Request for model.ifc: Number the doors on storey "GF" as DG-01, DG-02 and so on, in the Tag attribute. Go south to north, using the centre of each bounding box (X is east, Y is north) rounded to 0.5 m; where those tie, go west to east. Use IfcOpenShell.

First a look at what the model holds.

```python
import ifcopenshell
import ifcopenshell.util.element
import ifcopenshell.util.placement

model = ifcopenshell.open("model.ifc")
print(model.schema)
storey = next(s for s in model.by_type("IfcBuildingStorey") if s.Name == "GF")
doors = [e for e in ifcopenshell.util.element.get_decomposition(storey) if e.is_a("IfcDoor")]
for e in sorted(doors, key=lambda e: e.id()):
    origin = ifcopenshell.util.placement.get_local_placement(e.ObjectPlacement)[:3, 3]
    print(e.id(), e.Tag, e.Name, origin.round(2) + 0.0, sep=" | ")
```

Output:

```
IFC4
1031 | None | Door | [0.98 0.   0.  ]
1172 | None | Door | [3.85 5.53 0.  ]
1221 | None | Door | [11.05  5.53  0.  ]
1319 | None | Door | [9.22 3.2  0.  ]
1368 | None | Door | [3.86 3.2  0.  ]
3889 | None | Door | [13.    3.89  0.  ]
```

```python
import ifcopenshell
import ifcopenshell.geom
import ifcopenshell.util.element
import ifcopenshell.util.shape

model = ifcopenshell.open("model.ifc")
settings = ifcopenshell.geom.settings()
settings.set("use-world-coords", True)


def centre(element):
    shape = ifcopenshell.geom.create_shape(settings, element)
    return ifcopenshell.util.shape.get_bbox_centroid(shape.geometry)


storey = next(s for s in model.by_type("IfcBuildingStorey") if s.Name == "GF")
doors = [e for e in ifcopenshell.util.element.get_decomposition(storey) if e.is_a("IfcDoor")]

# Insertion points can sit at a corner or the storey origin, so sort by the geometry (in metres).
centres = {e: centre(e) for e in doors}
doors.sort(key=lambda e: (round(centres[e][1] / 0.5), centres[e][0]))

for i, e in enumerate(doors, start=1):
    number = f"DG-{i:02d}"
    e.Tag = number
    print(e.id(), number)

model.write("model-out.ifc")
```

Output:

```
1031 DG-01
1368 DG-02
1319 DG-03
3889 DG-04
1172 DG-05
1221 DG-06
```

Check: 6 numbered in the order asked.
